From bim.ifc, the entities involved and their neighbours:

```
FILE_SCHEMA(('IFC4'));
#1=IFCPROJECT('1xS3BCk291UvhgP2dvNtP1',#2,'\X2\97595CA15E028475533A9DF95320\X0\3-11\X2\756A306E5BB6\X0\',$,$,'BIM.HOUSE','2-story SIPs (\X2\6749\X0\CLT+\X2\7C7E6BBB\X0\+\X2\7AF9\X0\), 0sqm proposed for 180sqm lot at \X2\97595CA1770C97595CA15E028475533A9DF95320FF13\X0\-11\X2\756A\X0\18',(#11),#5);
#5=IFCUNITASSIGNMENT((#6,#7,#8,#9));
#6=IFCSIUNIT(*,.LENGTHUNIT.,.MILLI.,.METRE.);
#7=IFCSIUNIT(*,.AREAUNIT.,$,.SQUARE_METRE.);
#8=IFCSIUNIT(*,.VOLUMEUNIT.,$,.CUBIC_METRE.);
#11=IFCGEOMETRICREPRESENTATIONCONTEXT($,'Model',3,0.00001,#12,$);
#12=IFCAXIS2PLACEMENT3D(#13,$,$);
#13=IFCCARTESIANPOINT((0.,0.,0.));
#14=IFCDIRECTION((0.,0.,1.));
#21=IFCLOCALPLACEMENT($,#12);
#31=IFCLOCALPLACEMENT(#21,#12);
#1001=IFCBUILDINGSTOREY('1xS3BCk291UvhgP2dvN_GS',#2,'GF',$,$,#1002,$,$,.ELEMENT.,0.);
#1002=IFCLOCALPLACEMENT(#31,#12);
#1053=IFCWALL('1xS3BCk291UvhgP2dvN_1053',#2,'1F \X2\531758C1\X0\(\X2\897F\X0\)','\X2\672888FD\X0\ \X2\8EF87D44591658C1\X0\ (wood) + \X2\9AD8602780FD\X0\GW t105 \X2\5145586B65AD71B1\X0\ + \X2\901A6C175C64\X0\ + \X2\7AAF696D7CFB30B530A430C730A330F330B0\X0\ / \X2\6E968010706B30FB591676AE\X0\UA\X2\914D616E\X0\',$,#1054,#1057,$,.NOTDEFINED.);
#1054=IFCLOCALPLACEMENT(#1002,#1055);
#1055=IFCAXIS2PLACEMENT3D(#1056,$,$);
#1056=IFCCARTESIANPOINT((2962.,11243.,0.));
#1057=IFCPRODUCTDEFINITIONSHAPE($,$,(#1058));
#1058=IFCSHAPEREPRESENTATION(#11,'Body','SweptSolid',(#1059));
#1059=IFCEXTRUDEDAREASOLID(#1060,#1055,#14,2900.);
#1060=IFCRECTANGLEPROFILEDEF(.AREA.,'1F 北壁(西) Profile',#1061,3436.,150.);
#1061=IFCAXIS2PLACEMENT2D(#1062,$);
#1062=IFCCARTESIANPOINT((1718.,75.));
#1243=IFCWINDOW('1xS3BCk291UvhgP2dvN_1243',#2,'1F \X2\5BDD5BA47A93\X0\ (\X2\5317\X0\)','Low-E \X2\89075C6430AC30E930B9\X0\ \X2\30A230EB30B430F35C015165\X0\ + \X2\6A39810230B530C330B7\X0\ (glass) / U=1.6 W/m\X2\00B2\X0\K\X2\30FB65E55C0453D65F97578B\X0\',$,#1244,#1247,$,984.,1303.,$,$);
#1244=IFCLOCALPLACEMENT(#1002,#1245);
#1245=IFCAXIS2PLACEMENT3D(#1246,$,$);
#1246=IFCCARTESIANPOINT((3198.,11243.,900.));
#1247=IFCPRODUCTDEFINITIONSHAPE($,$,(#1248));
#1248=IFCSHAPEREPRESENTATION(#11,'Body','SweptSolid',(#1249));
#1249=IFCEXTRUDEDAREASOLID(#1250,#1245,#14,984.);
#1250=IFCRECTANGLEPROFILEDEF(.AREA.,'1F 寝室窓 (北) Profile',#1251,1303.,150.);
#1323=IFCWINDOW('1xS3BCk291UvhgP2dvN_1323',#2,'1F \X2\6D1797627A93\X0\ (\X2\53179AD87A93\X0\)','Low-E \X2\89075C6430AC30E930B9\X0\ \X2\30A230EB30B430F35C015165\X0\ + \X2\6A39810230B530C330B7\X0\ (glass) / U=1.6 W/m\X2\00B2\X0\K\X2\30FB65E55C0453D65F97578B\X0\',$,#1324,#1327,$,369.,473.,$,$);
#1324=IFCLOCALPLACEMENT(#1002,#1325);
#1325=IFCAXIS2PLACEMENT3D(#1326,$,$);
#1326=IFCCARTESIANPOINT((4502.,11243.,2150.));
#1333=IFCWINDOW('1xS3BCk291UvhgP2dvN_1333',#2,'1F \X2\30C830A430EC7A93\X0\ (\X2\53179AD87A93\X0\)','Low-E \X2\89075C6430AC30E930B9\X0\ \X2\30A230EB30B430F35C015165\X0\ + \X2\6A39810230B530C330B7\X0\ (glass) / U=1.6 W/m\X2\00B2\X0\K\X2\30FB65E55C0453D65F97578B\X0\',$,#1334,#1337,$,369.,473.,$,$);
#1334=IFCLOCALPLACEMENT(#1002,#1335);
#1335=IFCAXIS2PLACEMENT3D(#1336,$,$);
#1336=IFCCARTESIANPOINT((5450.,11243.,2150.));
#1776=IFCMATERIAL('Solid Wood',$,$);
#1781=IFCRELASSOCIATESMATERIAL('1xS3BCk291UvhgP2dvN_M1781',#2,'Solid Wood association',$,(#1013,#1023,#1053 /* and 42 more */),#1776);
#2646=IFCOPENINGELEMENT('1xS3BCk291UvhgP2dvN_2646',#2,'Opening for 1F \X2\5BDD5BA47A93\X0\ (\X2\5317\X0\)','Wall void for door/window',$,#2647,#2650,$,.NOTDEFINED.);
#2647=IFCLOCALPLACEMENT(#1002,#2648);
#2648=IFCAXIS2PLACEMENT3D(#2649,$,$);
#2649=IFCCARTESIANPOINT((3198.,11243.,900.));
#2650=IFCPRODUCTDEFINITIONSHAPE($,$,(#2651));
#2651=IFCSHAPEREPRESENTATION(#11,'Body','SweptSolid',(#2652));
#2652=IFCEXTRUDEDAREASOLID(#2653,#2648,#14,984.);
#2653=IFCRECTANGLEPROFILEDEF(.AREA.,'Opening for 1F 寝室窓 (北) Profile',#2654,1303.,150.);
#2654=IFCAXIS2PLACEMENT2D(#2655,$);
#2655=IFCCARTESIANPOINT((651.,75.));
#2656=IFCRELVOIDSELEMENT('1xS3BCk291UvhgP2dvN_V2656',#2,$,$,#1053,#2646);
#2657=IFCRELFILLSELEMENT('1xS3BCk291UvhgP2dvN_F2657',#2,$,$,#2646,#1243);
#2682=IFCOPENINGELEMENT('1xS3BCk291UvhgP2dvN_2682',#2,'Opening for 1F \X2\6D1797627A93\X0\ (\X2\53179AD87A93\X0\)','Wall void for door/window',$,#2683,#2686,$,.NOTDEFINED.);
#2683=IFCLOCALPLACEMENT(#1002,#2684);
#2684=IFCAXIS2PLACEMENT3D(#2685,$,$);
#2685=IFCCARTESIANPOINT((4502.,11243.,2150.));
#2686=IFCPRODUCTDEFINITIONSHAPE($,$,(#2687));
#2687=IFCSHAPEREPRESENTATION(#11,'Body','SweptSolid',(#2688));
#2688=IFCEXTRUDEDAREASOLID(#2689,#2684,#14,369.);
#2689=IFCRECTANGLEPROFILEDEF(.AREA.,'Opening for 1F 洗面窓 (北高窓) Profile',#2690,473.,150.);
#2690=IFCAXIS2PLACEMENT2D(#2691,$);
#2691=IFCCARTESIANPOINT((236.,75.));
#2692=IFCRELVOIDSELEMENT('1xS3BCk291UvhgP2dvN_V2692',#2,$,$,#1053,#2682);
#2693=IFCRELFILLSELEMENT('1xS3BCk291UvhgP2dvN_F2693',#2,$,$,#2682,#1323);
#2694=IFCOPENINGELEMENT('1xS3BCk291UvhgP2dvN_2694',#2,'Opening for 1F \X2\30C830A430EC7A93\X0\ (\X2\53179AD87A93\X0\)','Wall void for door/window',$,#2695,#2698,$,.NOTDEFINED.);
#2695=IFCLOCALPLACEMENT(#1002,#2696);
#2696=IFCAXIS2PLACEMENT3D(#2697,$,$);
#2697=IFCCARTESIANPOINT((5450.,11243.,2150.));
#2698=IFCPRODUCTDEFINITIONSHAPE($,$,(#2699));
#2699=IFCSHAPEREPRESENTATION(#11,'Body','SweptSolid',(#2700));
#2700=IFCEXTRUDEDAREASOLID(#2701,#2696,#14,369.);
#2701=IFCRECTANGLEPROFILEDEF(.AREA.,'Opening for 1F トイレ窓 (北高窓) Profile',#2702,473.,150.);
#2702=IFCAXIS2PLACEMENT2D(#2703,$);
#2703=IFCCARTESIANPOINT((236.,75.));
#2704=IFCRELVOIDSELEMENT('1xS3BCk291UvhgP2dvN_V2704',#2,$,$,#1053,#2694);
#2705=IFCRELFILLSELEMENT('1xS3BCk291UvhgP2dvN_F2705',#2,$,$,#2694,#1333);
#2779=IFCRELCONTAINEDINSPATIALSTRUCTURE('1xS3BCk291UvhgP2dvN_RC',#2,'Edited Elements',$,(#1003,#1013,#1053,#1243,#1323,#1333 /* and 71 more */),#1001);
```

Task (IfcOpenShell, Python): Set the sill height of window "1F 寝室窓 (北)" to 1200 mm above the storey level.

```python
import numpy as np
import ifcopenshell
import ifcopenshell.api.geometry
import ifcopenshell.geom
import ifcopenshell.util.element
import ifcopenshell.util.placement
import ifcopenshell.util.shape
import ifcopenshell.util.unit

model = ifcopenshell.open("bim.ifc")
unit_scale = ifcopenshell.util.unit.calculate_unit_scale(model)

window = model.by_id(1243)
opening = window.FillsVoids[0].RelatingOpeningElement
storey = ifcopenshell.util.element.get_container(window, ifc_class="IfcBuildingStorey")
level = ifcopenshell.util.placement.get_local_placement(storey.ObjectPlacement)[2, 3]

# The opening's origin need not be at the sill, so measure its lowest point.
shape = ifcopenshell.geom.create_shape(ifcopenshell.geom.settings(), opening)
bottom = ifcopenshell.util.shape.get_shape_bottom_elevation(shape, shape.geometry) / unit_scale
dz = level + 1200.0 - bottom

shift = np.array([0.0, 0.0, dz])
# The window is not placed relative to its opening, so move both.
for product in (opening, window):
    matrix = ifcopenshell.util.placement.get_local_placement(product.ObjectPlacement)
    matrix[:3, 3] += shift
    ifcopenshell.api.geometry.edit_object_placement(model, product=product, matrix=matrix, is_si=False)

print(f"moved by {dz * unit_scale:+.3f} m")

model.write("bim_edited.ifc")
```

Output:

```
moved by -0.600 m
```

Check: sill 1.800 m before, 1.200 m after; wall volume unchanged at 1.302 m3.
